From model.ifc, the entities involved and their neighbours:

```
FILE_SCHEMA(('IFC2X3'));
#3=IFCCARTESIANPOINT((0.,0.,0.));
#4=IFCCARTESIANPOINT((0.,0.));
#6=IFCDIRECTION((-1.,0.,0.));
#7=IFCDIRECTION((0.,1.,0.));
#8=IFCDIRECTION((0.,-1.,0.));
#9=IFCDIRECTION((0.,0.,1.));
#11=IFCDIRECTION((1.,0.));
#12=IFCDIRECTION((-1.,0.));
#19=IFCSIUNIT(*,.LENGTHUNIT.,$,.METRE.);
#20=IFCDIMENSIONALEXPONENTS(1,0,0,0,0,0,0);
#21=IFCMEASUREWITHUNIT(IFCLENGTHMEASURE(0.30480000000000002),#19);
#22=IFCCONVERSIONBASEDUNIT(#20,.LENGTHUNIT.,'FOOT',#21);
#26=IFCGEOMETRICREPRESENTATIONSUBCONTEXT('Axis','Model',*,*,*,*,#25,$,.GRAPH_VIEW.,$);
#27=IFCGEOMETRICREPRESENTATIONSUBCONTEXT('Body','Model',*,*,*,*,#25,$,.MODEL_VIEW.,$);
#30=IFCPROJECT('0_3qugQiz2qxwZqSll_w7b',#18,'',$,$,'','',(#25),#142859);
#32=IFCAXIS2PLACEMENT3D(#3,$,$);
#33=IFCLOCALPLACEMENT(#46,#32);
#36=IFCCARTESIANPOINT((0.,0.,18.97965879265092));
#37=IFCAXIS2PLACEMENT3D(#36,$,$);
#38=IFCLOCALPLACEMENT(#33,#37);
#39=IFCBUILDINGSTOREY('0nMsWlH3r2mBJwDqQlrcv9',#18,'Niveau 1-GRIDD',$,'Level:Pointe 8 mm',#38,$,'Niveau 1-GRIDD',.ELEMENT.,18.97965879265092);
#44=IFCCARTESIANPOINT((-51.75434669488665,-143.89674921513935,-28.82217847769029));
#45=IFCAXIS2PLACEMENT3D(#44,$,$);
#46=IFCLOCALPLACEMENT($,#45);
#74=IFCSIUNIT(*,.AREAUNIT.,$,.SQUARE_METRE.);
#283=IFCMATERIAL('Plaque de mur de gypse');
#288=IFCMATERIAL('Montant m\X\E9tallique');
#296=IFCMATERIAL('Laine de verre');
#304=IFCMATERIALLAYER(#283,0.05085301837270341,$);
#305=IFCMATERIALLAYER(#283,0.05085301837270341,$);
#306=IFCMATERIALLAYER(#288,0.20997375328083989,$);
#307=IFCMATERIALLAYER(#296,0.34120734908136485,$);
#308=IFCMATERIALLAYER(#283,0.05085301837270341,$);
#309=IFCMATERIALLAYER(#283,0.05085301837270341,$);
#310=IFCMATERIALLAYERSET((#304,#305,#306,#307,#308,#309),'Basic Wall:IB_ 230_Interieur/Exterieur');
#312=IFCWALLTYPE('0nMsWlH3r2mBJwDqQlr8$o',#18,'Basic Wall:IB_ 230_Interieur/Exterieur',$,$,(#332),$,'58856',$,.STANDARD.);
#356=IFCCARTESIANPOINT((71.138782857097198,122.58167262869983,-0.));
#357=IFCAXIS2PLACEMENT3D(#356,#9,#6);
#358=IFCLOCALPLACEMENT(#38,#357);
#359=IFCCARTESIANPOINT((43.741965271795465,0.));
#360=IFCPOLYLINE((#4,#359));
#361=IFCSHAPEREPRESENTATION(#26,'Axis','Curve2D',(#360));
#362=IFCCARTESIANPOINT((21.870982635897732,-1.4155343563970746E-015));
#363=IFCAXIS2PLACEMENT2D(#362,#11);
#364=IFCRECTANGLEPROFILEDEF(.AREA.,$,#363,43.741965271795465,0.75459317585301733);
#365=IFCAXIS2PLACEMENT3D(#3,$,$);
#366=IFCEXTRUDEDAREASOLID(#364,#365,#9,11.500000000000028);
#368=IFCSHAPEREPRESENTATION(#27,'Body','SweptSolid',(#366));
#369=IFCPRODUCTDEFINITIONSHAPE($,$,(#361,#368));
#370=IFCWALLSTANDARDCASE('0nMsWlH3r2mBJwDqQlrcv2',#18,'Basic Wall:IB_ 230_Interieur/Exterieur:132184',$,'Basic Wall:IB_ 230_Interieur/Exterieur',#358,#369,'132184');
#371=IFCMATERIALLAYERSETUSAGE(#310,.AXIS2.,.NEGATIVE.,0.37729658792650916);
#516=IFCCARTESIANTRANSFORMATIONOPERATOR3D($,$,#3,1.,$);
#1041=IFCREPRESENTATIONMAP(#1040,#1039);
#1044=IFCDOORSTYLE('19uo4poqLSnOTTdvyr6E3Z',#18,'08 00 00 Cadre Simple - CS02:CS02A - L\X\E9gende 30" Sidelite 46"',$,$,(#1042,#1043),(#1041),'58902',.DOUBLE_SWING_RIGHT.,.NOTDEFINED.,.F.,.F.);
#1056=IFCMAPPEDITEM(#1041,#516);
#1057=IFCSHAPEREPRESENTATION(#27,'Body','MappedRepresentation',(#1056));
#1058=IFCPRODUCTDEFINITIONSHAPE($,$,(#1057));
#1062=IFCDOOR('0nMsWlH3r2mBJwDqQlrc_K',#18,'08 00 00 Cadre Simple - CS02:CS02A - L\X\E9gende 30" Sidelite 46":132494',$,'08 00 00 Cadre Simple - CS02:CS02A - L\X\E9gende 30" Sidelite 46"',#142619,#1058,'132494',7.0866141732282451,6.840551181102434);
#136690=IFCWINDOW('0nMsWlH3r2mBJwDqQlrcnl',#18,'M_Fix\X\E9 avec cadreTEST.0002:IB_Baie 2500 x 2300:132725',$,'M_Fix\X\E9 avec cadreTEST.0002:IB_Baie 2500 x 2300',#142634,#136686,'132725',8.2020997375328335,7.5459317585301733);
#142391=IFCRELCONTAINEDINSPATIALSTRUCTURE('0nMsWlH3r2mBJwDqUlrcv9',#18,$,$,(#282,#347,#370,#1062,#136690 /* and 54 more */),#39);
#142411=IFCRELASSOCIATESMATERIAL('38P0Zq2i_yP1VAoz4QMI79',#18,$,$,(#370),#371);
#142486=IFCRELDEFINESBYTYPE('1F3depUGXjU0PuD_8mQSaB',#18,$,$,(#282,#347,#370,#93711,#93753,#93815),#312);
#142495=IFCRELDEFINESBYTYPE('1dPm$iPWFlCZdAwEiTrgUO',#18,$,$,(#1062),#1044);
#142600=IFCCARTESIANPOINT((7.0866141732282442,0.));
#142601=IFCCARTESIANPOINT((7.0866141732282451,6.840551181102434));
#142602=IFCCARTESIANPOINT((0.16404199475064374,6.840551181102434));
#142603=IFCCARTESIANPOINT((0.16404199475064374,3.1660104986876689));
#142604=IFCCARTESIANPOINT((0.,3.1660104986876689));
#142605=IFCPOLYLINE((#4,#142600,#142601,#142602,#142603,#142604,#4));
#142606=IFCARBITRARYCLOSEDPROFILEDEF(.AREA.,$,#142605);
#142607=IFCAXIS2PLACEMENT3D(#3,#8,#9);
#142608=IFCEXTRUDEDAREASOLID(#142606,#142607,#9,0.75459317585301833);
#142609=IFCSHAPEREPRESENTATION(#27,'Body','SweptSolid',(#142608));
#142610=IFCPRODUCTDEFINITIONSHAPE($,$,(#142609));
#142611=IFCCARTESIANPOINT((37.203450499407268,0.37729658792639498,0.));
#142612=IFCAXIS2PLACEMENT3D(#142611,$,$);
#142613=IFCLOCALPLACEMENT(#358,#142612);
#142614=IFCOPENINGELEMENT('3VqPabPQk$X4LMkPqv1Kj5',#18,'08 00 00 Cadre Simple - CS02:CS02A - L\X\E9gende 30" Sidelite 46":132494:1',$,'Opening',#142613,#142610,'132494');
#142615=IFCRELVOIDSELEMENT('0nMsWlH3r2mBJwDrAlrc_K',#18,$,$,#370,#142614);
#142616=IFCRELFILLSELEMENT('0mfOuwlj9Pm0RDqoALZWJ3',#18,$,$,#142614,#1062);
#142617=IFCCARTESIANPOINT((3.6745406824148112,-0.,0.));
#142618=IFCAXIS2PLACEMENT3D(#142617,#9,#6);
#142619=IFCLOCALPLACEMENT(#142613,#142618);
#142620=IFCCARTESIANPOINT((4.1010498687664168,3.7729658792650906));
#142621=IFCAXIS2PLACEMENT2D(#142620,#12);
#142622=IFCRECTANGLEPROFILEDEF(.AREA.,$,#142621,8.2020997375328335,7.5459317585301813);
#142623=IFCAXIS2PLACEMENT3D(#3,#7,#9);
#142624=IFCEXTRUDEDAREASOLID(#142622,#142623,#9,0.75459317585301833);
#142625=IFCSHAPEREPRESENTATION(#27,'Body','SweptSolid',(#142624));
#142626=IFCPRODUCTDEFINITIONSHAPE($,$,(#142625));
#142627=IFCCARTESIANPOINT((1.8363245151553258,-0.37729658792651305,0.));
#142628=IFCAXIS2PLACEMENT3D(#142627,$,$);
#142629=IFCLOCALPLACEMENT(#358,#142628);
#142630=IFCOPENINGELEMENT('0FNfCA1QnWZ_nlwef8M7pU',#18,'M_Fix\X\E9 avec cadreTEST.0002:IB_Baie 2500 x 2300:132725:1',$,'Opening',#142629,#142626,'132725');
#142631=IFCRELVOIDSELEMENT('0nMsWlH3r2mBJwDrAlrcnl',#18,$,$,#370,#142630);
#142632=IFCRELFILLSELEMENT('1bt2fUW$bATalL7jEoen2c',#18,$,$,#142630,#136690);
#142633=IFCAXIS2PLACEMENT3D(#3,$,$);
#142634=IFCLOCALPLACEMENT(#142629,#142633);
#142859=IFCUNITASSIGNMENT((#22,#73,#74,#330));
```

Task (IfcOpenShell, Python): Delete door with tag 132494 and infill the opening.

```python
import ifcopenshell
import ifcopenshell.api.feature
import ifcopenshell.api.root
import ifcopenshell.geom
import ifcopenshell.util.shape

model = ifcopenshell.open("model.ifc")
settings = ifcopenshell.geom.settings()


def volume(element):
    """Net volume in cubic metres, openings subtracted."""
    shape = ifcopenshell.geom.create_shape(settings, element)
    return ifcopenshell.util.shape.get_volume(shape.geometry)


door = model.by_guid("0nMsWlH3r2mBJwDqQlrc_K")
opening = door.FillsVoids[0].RelatingOpeningElement
wall = opening.VoidsElements[0].RelatingBuildingElement
before = volume(wall)

ifcopenshell.api.root.remove_product(model, product=door)
ifcopenshell.api.feature.remove_feature(model, feature=opening)

after = volume(wall)

print(f"wall volume {before:.3f} -> {after:.3f} m3")

model.write("model-out.ifc")
```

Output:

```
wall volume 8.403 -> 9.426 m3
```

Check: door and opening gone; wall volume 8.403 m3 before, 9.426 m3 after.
